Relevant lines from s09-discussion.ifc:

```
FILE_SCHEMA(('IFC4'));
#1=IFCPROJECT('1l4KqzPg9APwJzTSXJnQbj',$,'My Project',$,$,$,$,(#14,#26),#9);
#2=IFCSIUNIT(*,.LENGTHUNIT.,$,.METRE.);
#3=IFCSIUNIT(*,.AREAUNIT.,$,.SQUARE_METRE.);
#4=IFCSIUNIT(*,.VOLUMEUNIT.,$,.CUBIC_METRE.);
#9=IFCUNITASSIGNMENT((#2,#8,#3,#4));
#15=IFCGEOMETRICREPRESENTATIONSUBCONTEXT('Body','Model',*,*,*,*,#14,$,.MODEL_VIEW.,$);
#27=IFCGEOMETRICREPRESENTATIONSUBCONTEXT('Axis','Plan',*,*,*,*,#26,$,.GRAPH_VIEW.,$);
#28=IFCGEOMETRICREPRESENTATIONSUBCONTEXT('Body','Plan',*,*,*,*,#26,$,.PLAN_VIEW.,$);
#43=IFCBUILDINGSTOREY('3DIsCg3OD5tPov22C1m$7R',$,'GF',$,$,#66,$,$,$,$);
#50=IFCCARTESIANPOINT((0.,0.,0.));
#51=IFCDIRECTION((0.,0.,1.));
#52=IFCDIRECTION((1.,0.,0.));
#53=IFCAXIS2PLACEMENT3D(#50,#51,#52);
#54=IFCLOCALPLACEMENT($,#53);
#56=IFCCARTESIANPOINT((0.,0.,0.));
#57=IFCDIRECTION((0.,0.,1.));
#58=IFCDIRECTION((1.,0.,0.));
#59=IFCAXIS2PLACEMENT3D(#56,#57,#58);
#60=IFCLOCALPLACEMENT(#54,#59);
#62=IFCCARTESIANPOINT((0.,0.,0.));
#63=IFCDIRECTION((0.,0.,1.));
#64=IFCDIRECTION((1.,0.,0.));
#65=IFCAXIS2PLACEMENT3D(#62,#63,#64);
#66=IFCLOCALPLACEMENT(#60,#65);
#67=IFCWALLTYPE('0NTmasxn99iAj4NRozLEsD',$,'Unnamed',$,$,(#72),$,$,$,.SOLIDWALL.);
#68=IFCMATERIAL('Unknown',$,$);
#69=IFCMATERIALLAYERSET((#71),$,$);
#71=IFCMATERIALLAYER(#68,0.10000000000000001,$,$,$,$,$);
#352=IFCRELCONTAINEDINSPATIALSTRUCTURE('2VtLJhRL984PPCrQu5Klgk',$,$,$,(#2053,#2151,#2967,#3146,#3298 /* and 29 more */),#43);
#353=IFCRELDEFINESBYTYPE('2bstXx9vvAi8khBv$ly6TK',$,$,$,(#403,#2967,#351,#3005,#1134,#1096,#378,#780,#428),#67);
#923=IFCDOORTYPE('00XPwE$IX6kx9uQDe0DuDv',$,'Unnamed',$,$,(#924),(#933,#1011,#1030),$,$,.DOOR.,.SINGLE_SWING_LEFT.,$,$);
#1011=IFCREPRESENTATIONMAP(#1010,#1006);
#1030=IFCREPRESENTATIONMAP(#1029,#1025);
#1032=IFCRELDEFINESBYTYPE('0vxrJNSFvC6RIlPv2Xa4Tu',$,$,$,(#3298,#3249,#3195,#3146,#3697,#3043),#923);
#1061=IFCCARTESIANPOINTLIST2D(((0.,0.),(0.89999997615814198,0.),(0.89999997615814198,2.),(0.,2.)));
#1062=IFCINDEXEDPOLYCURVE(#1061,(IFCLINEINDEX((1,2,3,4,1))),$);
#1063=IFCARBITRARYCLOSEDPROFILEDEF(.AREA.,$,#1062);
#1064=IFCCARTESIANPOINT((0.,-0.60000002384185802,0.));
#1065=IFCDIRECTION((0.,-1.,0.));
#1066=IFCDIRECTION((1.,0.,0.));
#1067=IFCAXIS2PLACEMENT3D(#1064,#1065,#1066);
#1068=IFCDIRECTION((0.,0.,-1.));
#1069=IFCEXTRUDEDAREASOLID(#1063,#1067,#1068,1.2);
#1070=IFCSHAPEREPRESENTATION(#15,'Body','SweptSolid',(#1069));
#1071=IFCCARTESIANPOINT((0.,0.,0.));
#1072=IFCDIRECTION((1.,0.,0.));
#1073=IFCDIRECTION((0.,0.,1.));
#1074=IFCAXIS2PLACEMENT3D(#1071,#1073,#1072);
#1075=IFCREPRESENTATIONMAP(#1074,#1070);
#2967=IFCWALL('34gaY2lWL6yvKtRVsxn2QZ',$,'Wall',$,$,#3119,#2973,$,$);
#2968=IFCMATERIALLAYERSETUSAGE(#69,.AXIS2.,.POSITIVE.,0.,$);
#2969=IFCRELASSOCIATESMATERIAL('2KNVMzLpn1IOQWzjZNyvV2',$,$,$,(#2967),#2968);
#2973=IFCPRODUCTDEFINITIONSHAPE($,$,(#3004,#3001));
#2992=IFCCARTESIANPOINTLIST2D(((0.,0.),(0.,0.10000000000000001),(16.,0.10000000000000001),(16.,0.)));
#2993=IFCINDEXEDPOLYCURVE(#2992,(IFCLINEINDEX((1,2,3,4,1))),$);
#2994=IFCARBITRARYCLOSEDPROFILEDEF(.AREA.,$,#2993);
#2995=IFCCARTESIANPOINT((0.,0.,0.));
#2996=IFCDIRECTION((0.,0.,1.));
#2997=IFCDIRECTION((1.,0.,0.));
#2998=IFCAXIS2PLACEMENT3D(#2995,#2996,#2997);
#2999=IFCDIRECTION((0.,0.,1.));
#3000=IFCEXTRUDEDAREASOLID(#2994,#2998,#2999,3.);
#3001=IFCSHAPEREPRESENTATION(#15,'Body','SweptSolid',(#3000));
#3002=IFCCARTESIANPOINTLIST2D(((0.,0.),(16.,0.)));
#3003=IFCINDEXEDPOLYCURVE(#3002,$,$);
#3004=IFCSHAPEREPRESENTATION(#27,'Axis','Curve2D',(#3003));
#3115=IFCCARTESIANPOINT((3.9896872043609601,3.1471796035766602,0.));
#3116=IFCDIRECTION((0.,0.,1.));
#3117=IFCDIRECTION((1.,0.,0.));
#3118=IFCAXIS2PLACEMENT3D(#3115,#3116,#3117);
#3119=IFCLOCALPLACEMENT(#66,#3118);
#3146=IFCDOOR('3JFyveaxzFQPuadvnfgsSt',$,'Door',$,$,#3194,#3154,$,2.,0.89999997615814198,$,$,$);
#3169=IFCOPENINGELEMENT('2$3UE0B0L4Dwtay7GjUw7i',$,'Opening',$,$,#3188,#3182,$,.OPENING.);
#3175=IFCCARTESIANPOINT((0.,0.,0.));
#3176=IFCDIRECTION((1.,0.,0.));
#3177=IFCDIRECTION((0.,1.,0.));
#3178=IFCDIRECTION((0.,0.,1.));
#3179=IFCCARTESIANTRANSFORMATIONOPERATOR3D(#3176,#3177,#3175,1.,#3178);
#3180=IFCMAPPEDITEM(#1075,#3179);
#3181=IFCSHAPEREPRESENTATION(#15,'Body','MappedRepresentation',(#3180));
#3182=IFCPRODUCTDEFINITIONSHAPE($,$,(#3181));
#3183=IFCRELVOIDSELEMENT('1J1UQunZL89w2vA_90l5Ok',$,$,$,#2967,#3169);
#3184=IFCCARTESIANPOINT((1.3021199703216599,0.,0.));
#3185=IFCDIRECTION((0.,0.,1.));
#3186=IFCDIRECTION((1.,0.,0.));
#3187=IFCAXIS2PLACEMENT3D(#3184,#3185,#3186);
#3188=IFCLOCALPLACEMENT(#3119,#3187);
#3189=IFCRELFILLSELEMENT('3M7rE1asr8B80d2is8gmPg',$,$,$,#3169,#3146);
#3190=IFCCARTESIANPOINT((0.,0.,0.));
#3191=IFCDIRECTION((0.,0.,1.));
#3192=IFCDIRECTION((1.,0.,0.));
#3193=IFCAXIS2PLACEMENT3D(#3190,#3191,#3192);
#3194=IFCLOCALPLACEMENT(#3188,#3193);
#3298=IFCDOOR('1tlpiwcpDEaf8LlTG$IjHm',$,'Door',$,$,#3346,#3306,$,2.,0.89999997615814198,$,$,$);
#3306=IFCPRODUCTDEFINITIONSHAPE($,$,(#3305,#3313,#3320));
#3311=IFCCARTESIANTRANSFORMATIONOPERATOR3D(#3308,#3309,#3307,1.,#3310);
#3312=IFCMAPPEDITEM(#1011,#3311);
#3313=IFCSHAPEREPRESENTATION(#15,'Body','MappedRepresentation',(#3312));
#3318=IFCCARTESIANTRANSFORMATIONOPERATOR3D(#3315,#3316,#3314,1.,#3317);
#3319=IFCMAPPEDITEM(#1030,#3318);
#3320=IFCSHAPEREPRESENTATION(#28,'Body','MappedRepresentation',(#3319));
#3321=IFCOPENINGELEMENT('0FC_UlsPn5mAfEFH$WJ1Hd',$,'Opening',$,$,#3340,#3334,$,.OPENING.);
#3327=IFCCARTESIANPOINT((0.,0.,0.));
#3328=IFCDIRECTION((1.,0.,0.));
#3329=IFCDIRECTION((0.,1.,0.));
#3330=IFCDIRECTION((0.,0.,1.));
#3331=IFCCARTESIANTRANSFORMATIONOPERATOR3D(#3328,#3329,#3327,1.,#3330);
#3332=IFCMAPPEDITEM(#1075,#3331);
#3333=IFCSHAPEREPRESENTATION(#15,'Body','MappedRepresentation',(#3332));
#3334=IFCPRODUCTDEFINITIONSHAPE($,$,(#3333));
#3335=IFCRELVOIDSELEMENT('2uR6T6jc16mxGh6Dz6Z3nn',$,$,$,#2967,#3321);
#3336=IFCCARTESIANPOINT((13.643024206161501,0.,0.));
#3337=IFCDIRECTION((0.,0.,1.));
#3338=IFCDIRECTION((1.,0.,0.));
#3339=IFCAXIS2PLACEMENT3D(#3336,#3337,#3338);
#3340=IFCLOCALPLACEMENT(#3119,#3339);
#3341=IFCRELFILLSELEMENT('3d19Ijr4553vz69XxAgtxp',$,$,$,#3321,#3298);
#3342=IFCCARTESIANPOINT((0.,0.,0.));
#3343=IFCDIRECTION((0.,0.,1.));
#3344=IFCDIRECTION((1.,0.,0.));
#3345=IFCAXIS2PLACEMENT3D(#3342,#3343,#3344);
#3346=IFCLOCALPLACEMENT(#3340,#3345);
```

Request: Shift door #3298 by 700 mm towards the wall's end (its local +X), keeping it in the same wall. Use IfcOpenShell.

```python
import ifcopenshell
import ifcopenshell.api.geometry
import ifcopenshell.util.placement

model = ifcopenshell.open("s09-discussion.ifc")

door = model.by_id(3298)
opening = door.FillsVoids[0].RelatingOpeningElement
wall = opening.VoidsElements[0].RelatingBuildingElement

wall_matrix = ifcopenshell.util.placement.get_local_placement(wall.ObjectPlacement)
shift = wall_matrix[:3, 0] * 0.7
before = ifcopenshell.util.placement.get_local_placement(door.ObjectPlacement)[:3, 3].copy()

# The door is placed relative to its opening, so it follows when the opening moves.
matrix = ifcopenshell.util.placement.get_local_placement(opening.ObjectPlacement)
matrix[:3, 3] += shift
ifcopenshell.api.geometry.edit_object_placement(
    model, product=opening, matrix=matrix, is_si=False, should_transform_children=True
)

after = ifcopenshell.util.placement.get_local_placement(door.ObjectPlacement)[:3, 3]
print("door moved by", (after - before).round(3) + 0.0)

model.write("s09-discussion_updated.ifc")
```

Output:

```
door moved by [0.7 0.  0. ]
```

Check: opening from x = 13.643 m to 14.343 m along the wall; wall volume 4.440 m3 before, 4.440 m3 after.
